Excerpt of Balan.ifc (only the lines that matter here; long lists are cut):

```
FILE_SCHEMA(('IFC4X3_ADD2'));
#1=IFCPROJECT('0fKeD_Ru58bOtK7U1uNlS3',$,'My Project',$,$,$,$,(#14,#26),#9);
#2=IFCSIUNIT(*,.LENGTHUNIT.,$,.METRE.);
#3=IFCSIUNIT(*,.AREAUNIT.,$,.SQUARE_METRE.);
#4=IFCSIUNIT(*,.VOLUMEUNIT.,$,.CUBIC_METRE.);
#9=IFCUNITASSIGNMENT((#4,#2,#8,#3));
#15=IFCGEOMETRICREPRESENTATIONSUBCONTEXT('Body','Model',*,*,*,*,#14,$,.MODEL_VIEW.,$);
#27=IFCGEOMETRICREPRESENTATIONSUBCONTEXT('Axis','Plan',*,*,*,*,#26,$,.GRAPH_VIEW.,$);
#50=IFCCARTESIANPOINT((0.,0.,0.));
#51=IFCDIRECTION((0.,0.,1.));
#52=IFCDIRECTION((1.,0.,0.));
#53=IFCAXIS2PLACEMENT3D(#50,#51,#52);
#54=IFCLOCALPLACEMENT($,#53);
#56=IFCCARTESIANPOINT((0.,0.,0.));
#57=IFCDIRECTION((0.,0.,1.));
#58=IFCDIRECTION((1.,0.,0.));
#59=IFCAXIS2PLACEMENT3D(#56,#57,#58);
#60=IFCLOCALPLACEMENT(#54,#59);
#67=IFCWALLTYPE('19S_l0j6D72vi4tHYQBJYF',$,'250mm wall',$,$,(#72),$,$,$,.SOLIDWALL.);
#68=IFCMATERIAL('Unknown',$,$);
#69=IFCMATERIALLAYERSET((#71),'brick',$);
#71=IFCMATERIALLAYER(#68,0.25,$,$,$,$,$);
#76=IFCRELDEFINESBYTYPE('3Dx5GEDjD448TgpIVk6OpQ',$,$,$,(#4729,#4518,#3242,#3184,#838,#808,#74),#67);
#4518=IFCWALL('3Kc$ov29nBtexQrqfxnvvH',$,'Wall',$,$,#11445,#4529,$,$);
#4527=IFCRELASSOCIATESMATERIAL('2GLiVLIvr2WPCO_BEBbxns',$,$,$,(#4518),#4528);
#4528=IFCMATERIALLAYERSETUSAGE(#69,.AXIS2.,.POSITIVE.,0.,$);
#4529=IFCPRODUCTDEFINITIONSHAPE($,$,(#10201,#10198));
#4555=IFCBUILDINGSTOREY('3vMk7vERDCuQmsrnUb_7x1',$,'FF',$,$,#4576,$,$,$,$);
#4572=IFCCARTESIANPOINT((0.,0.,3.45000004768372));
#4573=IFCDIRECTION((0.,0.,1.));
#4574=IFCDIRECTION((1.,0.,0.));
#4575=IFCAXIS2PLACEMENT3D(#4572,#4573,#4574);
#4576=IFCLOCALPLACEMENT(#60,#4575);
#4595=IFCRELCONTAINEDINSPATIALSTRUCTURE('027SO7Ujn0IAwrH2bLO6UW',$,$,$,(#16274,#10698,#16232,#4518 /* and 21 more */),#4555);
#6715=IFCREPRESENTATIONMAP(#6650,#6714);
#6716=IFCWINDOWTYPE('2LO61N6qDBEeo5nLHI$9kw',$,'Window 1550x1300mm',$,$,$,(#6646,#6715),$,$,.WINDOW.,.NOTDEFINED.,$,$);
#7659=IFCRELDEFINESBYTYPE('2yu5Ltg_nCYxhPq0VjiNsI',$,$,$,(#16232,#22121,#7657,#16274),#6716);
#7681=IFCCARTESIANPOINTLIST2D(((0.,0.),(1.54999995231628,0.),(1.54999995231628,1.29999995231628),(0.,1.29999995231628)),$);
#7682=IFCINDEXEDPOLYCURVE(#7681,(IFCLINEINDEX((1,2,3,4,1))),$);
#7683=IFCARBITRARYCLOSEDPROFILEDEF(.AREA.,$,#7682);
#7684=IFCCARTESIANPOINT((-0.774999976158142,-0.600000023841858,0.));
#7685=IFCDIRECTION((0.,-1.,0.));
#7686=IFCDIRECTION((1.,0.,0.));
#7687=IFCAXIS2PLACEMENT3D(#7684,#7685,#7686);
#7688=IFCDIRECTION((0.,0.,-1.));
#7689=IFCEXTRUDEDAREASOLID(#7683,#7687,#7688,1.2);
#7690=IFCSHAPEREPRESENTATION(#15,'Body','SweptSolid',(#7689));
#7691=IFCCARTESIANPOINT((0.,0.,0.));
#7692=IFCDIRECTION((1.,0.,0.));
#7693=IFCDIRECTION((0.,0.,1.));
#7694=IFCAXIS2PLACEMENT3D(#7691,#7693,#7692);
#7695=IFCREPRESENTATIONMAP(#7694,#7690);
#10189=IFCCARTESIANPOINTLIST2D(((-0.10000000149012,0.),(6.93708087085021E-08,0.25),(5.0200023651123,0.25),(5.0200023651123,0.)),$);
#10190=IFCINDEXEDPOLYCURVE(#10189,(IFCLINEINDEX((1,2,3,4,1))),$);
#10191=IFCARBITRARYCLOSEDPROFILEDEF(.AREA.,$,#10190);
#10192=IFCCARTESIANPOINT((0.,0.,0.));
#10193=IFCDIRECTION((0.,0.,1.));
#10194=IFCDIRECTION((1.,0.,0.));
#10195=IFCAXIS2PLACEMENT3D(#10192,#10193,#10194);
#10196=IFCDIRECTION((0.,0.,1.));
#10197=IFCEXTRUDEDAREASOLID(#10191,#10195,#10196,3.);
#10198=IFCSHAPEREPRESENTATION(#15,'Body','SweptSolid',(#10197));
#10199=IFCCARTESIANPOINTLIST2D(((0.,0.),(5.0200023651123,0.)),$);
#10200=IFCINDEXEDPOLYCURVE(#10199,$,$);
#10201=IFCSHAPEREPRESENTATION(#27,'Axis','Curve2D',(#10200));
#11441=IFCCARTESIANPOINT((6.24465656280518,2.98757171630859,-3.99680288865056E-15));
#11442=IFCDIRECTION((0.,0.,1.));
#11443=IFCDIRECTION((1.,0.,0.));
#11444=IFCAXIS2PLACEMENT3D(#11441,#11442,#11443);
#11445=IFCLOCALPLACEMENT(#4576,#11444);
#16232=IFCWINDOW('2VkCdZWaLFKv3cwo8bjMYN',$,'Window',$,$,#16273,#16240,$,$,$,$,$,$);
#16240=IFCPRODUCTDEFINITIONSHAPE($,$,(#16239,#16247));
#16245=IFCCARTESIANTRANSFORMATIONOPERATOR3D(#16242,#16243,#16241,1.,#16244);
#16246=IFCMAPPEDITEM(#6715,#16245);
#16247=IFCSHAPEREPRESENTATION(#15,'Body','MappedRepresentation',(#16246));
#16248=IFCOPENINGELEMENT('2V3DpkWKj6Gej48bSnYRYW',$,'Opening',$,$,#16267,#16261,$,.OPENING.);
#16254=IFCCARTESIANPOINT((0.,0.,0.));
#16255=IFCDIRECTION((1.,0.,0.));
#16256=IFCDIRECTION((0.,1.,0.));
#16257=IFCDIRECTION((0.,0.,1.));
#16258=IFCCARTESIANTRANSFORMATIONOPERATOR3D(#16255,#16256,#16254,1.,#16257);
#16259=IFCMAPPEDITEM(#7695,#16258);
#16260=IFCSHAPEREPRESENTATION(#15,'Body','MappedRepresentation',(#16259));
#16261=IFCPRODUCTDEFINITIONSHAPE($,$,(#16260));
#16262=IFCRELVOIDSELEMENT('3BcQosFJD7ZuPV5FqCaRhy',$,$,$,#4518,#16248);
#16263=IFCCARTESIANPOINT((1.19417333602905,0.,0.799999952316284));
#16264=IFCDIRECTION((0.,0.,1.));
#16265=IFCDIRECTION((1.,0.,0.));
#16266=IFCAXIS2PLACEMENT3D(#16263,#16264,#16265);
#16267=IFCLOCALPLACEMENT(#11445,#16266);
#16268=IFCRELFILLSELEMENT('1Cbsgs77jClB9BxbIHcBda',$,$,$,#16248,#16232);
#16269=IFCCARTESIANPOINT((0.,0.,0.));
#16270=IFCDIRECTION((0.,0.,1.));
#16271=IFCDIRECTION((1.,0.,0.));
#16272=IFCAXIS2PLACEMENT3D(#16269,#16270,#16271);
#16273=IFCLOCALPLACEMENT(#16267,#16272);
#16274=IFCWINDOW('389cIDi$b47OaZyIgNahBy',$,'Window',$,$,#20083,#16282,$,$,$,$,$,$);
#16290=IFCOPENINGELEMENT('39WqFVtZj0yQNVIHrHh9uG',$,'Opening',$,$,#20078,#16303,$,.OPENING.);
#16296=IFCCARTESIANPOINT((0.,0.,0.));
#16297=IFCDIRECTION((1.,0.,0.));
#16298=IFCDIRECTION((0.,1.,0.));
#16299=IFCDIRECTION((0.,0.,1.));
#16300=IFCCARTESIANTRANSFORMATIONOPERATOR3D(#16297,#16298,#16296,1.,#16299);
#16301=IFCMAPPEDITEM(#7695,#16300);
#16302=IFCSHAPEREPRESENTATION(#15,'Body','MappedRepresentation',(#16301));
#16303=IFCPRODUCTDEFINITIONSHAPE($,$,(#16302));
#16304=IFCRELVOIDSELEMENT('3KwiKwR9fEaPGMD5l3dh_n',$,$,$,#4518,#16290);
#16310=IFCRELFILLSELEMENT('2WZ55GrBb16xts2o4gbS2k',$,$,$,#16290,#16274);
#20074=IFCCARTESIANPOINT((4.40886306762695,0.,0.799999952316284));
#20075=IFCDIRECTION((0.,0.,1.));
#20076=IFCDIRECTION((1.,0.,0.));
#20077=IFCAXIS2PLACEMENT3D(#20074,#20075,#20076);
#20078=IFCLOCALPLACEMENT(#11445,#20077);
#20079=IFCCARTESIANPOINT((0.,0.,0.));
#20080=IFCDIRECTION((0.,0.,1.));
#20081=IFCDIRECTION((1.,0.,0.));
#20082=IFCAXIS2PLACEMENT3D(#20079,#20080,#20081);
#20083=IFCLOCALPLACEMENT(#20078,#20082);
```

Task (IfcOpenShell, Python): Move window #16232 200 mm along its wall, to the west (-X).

```python
import ifcopenshell
import ifcopenshell.api.geometry
import ifcopenshell.util.placement
import ifcopenshell.util.unit

model = ifcopenshell.open("Balan.ifc")
unit_scale = ifcopenshell.util.unit.calculate_unit_scale(model)

window = model.by_id(16232)
opening = window.FillsVoids[0].RelatingOpeningElement
wall = opening.VoidsElements[0].RelatingBuildingElement

wall_matrix = ifcopenshell.util.placement.get_local_placement(wall.ObjectPlacement)
shift = wall_matrix[:3, 0] * -0.2 / unit_scale
before = ifcopenshell.util.placement.get_local_placement(window.ObjectPlacement)[:3, 3].copy()

# The window is placed relative to its opening, so it follows when the opening moves.
matrix = ifcopenshell.util.placement.get_local_placement(opening.ObjectPlacement)
matrix[:3, 3] += shift
ifcopenshell.api.geometry.edit_object_placement(
    model, product=opening, matrix=matrix, is_si=False, should_transform_children=True
)

after = ifcopenshell.util.placement.get_local_placement(window.ObjectPlacement)[:3, 3]
print("window moved by", (after - before).round(3) + 0.0)

model.write("Balan_edited.ifc")
```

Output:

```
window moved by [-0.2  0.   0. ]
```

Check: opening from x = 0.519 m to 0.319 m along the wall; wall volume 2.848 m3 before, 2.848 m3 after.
